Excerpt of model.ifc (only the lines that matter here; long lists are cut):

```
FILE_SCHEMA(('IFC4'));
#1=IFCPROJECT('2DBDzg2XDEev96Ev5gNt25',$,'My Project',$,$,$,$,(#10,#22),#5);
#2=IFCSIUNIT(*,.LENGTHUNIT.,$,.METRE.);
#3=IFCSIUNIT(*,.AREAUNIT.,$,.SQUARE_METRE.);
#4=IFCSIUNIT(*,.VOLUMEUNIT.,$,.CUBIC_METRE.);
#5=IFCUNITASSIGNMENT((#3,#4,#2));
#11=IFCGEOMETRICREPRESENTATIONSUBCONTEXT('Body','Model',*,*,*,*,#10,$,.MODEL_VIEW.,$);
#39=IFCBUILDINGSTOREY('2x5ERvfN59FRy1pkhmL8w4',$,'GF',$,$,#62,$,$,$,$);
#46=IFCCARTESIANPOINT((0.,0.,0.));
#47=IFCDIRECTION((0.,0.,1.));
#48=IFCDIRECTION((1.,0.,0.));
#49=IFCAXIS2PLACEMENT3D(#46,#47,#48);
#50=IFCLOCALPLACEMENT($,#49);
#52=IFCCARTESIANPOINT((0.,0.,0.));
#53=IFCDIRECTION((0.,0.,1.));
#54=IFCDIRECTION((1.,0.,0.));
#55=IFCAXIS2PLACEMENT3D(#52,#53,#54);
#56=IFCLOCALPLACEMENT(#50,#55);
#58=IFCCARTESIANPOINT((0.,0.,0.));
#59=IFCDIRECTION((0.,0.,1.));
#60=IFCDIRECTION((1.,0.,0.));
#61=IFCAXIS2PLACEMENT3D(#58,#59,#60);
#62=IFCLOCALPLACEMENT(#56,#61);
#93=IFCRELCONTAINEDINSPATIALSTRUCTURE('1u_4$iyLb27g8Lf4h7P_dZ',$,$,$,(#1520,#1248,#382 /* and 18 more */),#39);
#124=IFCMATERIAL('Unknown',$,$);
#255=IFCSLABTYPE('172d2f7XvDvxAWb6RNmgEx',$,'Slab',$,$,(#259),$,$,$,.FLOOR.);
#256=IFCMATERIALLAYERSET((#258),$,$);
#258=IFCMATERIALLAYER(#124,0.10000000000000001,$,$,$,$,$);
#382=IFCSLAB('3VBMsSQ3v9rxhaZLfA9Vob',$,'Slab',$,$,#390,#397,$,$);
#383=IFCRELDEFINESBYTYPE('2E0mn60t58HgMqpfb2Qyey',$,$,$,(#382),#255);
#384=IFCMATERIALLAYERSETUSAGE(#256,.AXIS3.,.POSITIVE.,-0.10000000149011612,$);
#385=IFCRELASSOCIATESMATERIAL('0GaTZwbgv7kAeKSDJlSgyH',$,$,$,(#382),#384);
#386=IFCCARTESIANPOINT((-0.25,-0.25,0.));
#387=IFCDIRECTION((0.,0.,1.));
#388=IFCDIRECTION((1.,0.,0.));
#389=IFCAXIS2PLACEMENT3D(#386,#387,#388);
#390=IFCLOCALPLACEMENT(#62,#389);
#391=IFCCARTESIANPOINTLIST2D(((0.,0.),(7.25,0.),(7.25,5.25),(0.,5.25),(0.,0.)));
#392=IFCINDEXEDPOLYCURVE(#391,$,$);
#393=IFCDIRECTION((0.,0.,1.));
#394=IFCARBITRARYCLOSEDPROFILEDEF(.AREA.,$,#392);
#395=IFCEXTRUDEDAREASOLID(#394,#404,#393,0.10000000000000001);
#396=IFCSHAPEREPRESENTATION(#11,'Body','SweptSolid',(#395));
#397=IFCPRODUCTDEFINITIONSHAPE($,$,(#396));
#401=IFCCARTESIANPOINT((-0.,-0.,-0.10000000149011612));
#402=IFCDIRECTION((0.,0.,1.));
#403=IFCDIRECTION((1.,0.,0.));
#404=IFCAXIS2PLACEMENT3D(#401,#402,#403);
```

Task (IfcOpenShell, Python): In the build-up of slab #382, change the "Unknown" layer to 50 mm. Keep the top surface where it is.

```python
import ifcopenshell
import ifcopenshell.util.element
import ifcopenshell.util.representation
import ifcopenshell.util.unit

model = ifcopenshell.open("model.ifc")
unit_scale = ifcopenshell.util.unit.calculate_unit_scale(model)

layer_set = model.by_id(256)
layer = next(l for l in layer_set.MaterialLayers if l.Material and l.Material.Name == "Unknown")
change = 0.05 / unit_scale - layer.LayerThickness
layer.LayerThickness += change

# Geometry does not follow the layer set by itself.
slabs = [e for e in ifcopenshell.util.element.get_elements_by_material(model, layer_set) if e.is_a("IfcSlab")]
for slab in sorted(slabs, key=lambda e: e.id()):
    body = ifcopenshell.util.representation.get_representation(slab, "Model", "Body")
    solid = body.Items[0]
    old_depth = solid.Depth
    solid.Depth += change
    # Extruded upwards: lower the start of the extrusion so the top stays.
    x, y, z = solid.Position.Location.Coordinates
    solid.Position.Location = model.createIfcCartesianPoint((x, y, z - change))
    print(slab.id(), f"{old_depth:g} -> {solid.Depth:g}")

# The layers are counted up from the underside, which has moved.
for usage in {ifcopenshell.util.element.get_material(slab) for slab in slabs}:
    usage.OffsetFromReferenceLine -= change

model.write("model_v2.ifc")
```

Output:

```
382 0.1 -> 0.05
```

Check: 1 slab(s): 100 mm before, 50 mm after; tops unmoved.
